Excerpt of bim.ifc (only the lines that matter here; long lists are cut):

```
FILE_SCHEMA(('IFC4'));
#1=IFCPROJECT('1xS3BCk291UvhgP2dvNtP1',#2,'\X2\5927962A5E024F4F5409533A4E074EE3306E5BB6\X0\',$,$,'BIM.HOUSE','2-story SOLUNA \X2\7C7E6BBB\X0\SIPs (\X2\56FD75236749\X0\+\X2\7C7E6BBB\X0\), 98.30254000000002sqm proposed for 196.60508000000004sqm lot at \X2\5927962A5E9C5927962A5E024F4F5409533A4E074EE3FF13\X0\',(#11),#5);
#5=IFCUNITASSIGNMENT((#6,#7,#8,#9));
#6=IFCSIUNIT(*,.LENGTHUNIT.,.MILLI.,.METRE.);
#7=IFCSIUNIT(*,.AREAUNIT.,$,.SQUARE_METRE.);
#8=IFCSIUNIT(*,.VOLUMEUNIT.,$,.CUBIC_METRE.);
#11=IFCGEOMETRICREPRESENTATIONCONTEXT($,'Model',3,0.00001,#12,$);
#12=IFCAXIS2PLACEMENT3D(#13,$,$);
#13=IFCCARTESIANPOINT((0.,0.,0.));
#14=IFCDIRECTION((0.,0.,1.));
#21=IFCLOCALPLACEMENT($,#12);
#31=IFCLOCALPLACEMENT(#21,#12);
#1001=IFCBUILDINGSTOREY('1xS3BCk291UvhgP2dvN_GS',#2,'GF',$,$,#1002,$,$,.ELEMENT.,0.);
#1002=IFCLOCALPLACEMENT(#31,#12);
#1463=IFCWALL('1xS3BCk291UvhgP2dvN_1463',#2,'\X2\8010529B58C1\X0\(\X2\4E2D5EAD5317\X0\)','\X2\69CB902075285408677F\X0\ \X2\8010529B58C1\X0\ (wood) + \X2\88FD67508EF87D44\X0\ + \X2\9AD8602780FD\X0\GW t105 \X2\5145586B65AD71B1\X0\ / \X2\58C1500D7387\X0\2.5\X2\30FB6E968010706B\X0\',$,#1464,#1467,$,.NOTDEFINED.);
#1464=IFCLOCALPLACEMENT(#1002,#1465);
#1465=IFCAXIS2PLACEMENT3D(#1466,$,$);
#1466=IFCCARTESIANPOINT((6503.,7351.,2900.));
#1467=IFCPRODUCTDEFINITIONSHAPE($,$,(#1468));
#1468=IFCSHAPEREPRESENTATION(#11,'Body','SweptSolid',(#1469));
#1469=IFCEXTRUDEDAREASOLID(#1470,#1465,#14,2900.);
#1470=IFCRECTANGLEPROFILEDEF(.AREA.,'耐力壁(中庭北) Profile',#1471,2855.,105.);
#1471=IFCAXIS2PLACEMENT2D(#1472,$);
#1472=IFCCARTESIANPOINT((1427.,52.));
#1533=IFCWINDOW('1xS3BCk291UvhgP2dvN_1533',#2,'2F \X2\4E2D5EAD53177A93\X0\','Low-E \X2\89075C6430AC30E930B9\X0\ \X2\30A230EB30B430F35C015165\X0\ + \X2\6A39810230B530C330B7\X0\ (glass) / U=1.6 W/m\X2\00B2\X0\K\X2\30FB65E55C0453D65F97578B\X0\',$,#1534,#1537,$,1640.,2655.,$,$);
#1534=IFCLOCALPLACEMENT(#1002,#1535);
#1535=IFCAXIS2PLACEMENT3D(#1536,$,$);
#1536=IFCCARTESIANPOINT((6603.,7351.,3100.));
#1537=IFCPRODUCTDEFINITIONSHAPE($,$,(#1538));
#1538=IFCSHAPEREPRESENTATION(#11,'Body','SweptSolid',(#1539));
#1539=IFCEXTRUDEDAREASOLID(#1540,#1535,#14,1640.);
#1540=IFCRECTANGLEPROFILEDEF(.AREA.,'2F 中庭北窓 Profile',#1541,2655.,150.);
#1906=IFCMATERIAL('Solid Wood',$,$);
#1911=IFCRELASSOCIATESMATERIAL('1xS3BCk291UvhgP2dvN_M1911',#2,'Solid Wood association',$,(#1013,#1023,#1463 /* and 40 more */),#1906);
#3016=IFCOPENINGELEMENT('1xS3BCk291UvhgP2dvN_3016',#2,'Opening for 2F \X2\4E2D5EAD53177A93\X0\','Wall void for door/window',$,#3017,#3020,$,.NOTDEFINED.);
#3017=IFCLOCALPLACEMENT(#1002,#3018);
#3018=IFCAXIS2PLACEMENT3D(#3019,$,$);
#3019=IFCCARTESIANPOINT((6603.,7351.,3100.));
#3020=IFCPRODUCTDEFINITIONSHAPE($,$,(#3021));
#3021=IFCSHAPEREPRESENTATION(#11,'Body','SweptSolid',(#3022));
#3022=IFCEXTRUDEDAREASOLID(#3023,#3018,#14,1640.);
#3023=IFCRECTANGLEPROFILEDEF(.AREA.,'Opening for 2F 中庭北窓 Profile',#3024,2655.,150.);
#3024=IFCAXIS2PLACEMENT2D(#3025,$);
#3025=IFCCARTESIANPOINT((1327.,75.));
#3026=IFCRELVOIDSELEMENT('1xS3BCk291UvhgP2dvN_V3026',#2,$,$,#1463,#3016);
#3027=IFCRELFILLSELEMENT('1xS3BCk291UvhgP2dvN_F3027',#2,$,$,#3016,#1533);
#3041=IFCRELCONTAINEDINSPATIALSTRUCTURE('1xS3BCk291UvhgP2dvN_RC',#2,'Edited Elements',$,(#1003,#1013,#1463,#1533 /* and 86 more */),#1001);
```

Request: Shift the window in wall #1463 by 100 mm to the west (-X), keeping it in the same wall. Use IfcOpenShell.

```python
import ifcopenshell
import ifcopenshell.api.geometry
import ifcopenshell.util.placement
import ifcopenshell.util.unit

model = ifcopenshell.open("bim.ifc")
unit_scale = ifcopenshell.util.unit.calculate_unit_scale(model)

window = model.by_guid("1xS3BCk291UvhgP2dvN_1533")
opening = window.FillsVoids[0].RelatingOpeningElement
wall = opening.VoidsElements[0].RelatingBuildingElement

wall_matrix = ifcopenshell.util.placement.get_local_placement(wall.ObjectPlacement)
shift = wall_matrix[:3, 0] * -0.1 / unit_scale
before = ifcopenshell.util.placement.get_local_placement(window.ObjectPlacement)[:3, 3].copy()

# The window is not placed relative to its opening, so move both.
for product in (opening, window):
    matrix = ifcopenshell.util.placement.get_local_placement(product.ObjectPlacement)
    matrix[:3, 3] += shift
    ifcopenshell.api.geometry.edit_object_placement(model, product=product, matrix=matrix, is_si=False)

after = ifcopenshell.util.placement.get_local_placement(window.ObjectPlacement)[:3, 3]
print("window moved by", (after - before).round(3) + 0.0)

model.write("bim-out.ifc")
```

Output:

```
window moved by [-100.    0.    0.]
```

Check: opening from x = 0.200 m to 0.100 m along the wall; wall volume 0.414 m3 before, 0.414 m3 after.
